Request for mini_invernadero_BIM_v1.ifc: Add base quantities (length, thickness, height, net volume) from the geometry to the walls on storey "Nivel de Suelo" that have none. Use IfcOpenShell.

First a look at what the model holds.

```python
import ifcopenshell
import ifcopenshell.util.element
import ifcopenshell.util.unit

model = ifcopenshell.open("mini_invernadero_BIM_v1.ifc")
print(model.schema)
for unit_type in ("LENGTHUNIT", "AREAUNIT", "VOLUMEUNIT"):
    print(unit_type, ifcopenshell.util.unit.calculate_unit_scale(model, unit_type))
storey = next(s for s in model.by_type("IfcBuildingStorey") if s.Name == "Nivel de Suelo")
walls = [e for e in ifcopenshell.util.element.get_decomposition(storey) if e.is_a("IfcWall")]
for e in sorted(walls, key=lambda e: e.id()):
    print(e.id(), e.is_a(), e.Name, list(ifcopenshell.util.element.get_psets(e, qtos_only=True)), sep=" | ")
```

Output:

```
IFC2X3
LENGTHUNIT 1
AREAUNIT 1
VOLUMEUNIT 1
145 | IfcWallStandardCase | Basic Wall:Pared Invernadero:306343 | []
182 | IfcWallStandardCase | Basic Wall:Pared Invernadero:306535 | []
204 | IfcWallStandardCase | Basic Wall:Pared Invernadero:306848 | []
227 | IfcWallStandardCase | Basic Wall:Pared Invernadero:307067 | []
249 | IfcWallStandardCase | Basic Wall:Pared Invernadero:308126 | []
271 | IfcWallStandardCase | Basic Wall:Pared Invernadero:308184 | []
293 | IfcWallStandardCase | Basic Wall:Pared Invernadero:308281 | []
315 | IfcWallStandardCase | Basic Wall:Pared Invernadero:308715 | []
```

```python
import ifcopenshell
import ifcopenshell.api.pset
import ifcopenshell.geom
import ifcopenshell.util.element
import ifcopenshell.util.shape
import ifcopenshell.util.unit

model = ifcopenshell.open("mini_invernadero_BIM_v1.ifc")
unit_scale = ifcopenshell.util.unit.calculate_unit_scale(model)
volume_scale = ifcopenshell.util.unit.calculate_unit_scale(model, "VOLUMEUNIT")
settings = ifcopenshell.geom.settings()

storey = next(s for s in model.by_type("IfcBuildingStorey") if s.Name == "Nivel de Suelo")
walls = [e for e in ifcopenshell.util.element.get_decomposition(storey) if e.is_a("IfcWall")]

for e in sorted(walls, key=lambda e: e.id()):
    if ifcopenshell.util.element.get_psets(e, qtos_only=True, should_inherit=False):
        continue
    # Geometry comes back in metres, in the element's own axes.
    shape = ifcopenshell.geom.create_shape(settings, e)
    values = {
        "Length": ifcopenshell.util.shape.get_x(shape.geometry) / unit_scale,
        "Width": ifcopenshell.util.shape.get_y(shape.geometry) / unit_scale,
        "Height": ifcopenshell.util.shape.get_z(shape.geometry) / unit_scale,
        "NetVolume": ifcopenshell.util.shape.get_volume(shape.geometry) / volume_scale,
    }
    qto = ifcopenshell.api.pset.add_qto(model, product=e, name="BaseQuantities")
    ifcopenshell.api.pset.edit_qto(model, qto=qto, properties=values)
    print(e.id(), {k: round(v, 3) for k, v in values.items()})

model.write("mini_invernadero_BIM_v1_updated.ifc")
```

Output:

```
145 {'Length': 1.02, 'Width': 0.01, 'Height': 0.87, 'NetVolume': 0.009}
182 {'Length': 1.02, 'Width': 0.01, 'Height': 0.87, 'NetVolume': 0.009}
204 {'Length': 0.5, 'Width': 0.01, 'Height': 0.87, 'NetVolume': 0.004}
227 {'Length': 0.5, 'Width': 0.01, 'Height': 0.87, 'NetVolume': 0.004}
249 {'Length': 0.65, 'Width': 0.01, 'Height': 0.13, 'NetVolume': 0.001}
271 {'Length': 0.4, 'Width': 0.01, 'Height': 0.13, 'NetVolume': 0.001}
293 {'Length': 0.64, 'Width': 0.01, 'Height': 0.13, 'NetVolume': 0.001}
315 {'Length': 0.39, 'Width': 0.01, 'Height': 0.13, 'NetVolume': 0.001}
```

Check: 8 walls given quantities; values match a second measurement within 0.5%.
